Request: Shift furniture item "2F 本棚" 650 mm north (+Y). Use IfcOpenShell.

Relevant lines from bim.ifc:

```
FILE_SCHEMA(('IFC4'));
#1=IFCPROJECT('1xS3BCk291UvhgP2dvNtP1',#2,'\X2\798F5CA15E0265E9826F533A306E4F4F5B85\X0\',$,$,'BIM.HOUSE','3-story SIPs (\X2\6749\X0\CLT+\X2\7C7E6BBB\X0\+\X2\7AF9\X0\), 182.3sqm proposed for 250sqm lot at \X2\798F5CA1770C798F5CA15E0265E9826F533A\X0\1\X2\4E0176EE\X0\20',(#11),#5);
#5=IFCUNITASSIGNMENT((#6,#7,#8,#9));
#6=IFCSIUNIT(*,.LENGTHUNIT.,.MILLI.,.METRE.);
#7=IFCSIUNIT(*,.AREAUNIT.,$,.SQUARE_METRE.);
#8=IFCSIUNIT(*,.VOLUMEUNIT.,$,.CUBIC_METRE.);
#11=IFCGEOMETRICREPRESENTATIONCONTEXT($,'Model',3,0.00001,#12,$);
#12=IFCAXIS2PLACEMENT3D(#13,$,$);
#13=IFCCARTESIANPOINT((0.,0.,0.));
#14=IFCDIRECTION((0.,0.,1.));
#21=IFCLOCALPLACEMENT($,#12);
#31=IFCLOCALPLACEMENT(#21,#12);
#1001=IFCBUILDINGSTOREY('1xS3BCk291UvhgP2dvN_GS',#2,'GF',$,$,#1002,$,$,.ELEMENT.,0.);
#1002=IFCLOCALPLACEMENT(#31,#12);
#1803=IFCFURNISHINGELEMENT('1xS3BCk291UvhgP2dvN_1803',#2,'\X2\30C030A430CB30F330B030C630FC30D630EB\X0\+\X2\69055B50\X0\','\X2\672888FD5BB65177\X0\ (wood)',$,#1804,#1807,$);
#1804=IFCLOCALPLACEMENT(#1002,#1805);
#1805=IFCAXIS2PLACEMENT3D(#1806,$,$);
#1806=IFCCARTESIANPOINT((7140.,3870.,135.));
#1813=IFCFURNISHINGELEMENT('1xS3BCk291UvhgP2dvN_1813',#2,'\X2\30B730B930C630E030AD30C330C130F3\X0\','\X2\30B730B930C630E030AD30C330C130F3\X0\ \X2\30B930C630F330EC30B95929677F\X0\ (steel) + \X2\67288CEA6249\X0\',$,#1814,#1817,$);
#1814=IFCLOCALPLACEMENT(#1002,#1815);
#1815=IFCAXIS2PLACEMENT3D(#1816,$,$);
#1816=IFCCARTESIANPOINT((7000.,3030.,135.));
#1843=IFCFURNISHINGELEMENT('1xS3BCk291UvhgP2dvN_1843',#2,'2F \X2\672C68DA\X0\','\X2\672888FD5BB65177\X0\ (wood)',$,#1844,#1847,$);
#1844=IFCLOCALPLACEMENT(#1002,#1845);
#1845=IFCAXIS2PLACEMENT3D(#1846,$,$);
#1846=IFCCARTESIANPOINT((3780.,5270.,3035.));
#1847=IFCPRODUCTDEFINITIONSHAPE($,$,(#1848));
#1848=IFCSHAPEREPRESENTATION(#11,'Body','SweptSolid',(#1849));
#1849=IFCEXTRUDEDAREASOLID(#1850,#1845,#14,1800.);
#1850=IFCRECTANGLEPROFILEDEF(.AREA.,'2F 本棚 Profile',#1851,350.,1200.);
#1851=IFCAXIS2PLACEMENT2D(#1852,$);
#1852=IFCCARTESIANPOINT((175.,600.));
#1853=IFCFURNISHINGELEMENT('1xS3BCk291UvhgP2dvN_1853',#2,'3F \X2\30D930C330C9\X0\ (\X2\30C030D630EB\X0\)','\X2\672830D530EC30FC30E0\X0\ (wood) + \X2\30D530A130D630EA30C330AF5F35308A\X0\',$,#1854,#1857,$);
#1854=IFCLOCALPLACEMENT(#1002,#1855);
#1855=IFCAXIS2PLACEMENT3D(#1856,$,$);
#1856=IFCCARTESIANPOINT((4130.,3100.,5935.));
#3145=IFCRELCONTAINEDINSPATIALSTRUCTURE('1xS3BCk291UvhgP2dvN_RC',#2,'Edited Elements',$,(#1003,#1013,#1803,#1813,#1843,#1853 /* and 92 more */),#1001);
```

```python
import ifcopenshell
import ifcopenshell.api.geometry
import ifcopenshell.util.placement
import ifcopenshell.util.unit

model = ifcopenshell.open("bim.ifc")
unit_scale = ifcopenshell.util.unit.calculate_unit_scale(model)

item = model.by_id(1843)
matrix = ifcopenshell.util.placement.get_local_placement(item.ObjectPlacement)
matrix[1, 3] += 0.65 / unit_scale
ifcopenshell.api.geometry.edit_object_placement(model, product=item, matrix=matrix, is_si=False)

print(ifcopenshell.util.placement.get_local_placement(item.ObjectPlacement).round(3) + 0.0)

model.write("bim_v2.ifc")
```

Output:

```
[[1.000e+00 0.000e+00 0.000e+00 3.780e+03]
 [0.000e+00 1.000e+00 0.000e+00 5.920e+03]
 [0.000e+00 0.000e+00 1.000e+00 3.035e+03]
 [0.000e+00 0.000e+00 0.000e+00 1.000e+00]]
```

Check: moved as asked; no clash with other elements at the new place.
